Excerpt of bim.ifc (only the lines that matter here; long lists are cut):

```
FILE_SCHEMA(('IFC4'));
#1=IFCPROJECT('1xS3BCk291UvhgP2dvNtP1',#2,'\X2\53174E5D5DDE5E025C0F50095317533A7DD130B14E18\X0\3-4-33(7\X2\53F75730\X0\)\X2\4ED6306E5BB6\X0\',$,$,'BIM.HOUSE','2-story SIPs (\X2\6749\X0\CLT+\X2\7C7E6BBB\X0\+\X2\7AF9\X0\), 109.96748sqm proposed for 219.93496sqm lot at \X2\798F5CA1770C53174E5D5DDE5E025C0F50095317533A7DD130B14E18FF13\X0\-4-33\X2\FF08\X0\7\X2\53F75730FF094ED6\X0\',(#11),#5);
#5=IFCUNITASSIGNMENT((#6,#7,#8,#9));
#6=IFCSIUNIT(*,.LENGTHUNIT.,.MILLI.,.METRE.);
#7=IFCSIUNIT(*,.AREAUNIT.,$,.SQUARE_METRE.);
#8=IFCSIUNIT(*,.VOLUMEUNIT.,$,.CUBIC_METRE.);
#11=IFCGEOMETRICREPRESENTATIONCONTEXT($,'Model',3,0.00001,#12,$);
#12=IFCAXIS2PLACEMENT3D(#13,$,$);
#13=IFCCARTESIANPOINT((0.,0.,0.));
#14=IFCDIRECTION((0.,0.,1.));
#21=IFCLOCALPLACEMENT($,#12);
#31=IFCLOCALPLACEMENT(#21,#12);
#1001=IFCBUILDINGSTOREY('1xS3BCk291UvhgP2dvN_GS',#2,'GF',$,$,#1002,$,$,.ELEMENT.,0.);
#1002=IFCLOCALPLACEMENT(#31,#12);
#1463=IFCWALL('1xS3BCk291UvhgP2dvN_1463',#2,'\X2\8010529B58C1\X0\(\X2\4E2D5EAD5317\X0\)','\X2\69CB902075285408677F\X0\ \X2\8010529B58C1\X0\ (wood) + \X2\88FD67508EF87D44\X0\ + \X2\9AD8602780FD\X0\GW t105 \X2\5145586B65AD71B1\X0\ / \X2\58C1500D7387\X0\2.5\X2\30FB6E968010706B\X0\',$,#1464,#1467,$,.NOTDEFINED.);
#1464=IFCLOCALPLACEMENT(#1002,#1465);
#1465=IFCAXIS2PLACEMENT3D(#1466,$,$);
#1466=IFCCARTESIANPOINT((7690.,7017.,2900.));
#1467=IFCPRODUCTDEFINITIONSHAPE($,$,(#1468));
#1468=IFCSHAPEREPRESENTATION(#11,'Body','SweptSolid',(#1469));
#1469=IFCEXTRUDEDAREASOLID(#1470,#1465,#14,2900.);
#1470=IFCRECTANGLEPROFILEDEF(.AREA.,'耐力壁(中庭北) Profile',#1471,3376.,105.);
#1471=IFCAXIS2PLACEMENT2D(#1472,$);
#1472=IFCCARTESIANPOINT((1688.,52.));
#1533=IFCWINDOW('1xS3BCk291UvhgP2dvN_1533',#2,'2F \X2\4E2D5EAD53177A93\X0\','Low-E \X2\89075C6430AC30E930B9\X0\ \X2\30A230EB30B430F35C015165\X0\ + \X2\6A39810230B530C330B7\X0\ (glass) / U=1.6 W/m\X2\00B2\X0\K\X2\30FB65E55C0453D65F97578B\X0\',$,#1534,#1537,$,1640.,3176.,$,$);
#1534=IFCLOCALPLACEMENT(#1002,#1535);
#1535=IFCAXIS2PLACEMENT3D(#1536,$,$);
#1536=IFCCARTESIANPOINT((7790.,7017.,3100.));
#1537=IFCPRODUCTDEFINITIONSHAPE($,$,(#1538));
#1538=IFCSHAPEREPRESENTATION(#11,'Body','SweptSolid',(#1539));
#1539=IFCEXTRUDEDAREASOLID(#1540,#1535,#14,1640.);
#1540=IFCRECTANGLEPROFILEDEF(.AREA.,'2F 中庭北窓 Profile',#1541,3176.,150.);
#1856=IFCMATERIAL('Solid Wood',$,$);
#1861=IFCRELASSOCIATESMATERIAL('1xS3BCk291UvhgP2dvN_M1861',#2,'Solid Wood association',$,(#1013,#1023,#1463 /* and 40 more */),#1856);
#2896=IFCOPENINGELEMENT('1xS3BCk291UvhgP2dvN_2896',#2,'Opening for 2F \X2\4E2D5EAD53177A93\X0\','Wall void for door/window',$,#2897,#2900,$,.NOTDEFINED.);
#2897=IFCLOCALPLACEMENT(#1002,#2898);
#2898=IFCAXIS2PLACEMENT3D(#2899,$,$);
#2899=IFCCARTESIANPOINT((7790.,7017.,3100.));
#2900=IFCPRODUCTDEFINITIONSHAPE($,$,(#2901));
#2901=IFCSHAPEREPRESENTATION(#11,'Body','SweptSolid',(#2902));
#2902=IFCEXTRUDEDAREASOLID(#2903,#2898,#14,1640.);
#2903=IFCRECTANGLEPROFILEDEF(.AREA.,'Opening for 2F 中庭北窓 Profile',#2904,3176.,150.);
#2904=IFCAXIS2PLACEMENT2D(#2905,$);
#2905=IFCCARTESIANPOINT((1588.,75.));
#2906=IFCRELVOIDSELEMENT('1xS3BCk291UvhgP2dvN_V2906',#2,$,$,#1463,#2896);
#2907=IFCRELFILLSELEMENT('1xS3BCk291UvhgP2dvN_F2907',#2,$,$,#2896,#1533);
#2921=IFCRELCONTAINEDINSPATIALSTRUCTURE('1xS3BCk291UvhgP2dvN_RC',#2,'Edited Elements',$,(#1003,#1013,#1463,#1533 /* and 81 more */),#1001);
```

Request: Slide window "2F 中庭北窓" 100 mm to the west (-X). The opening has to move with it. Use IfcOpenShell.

```python
import ifcopenshell
import ifcopenshell.api.geometry
import ifcopenshell.util.placement

model = ifcopenshell.open("bim.ifc")

window = model.by_guid("1xS3BCk291UvhgP2dvN_1533")
opening = window.FillsVoids[0].RelatingOpeningElement
wall = opening.VoidsElements[0].RelatingBuildingElement

wall_matrix = ifcopenshell.util.placement.get_local_placement(wall.ObjectPlacement)
shift = wall_matrix[:3, 0] * -100.0
before = ifcopenshell.util.placement.get_local_placement(window.ObjectPlacement)[:3, 3].copy()

# The window is not placed relative to its opening, so move both.
for product in (opening, window):
    matrix = ifcopenshell.util.placement.get_local_placement(product.ObjectPlacement)
    matrix[:3, 3] += shift
    ifcopenshell.api.geometry.edit_object_placement(model, product=product, matrix=matrix, is_si=False)

after = ifcopenshell.util.placement.get_local_placement(window.ObjectPlacement)[:3, 3]
print("window moved by", (after - before).round(3) + 0.0)

model.write("bim_v2.ifc")
```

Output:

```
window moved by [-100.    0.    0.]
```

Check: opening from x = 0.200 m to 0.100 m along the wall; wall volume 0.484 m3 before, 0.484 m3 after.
